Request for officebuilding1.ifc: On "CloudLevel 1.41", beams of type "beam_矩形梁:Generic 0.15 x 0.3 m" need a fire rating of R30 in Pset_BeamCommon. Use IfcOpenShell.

First a look at what the model holds.

```python
import ifcopenshell
import ifcopenshell.util.element

model = ifcopenshell.open("officebuilding1.ifc")
print(model.schema)
storey = next(s for s in model.by_type("IfcBuildingStorey") if s.Name == "CloudLevel 1.41")
beams = [e for e in ifcopenshell.util.element.get_decomposition(storey) if e.is_a("IfcBeam")]
seen = {}
for e in beams:
    element_type = ifcopenshell.util.element.get_type(e)
    key = (element_type.Name if element_type != e and element_type else None, ifcopenshell.util.element.get_pset(e, "Pset_BeamCommon", "FireRating"))
    seen[key] = seen.get(key, 0) + 1
for (name, value), count in sorted(seen.items(), key=str):
    print(count, "x", name, "|", value)
```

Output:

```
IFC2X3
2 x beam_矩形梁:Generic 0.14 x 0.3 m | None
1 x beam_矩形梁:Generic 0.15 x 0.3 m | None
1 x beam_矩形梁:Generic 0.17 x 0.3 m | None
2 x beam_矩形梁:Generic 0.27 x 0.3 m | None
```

```python
import ifcopenshell
import ifcopenshell.api.pset
import ifcopenshell.util.element

model = ifcopenshell.open("officebuilding1.ifc")

storey = next(s for s in model.by_type("IfcBuildingStorey") if s.Name == "CloudLevel 1.41")
beams = [e for e in ifcopenshell.util.element.get_decomposition(storey) if e.is_a("IfcBeam")]

count = 0
for e in beams:
    element_type = ifcopenshell.util.element.get_type(e)
    if element_type in (None, e) or element_type.Name != "beam_矩形梁:Generic 0.15 x 0.3 m":
        continue
    # add_pset returns the element's existing set when there is one.
    pset = ifcopenshell.api.pset.add_pset(model, product=e, name="Pset_BeamCommon")
    ifcopenshell.api.pset.edit_pset(model, pset=pset, properties={"FireRating": "R30"})
    count += 1

print(count, "beams updated")

model.write("officebuilding1_edited.ifc")
```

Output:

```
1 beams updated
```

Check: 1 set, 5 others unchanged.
